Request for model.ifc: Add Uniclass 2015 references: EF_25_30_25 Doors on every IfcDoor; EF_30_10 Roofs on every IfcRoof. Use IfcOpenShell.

First a look at what the model holds.

```python
import ifcopenshell

model = ifcopenshell.open("model.ifc")
print(model.schema)
print("classifications:", [c.Name for c in model.by_type("IfcClassification")])
for ifc_class in ("IfcDoor", "IfcRoof", "IfcStair", "IfcWall", "IfcWindow"):
    print(ifc_class, len(model.by_type(ifc_class)))
```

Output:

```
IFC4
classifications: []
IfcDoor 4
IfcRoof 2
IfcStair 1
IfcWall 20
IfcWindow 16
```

```python
import ifcopenshell
import ifcopenshell.api.classification

model = ifcopenshell.open("model.ifc")

system = ifcopenshell.api.classification.add_classification(model, classification="Uniclass 2015")

codes = {
    "IfcDoor": ("EF_25_30_25", "Doors"),
    "IfcRoof": ("EF_30_10", "Roofs"),
}
for ifc_class, (code, name) in codes.items():
    products = model.by_type(ifc_class)
    ifcopenshell.api.classification.add_reference(
        model, products=products, classification=system, identification=code, name=name
    )
    print(code, len(products))

model.write("model-out.ifc")
```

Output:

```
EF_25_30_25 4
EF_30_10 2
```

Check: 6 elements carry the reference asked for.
